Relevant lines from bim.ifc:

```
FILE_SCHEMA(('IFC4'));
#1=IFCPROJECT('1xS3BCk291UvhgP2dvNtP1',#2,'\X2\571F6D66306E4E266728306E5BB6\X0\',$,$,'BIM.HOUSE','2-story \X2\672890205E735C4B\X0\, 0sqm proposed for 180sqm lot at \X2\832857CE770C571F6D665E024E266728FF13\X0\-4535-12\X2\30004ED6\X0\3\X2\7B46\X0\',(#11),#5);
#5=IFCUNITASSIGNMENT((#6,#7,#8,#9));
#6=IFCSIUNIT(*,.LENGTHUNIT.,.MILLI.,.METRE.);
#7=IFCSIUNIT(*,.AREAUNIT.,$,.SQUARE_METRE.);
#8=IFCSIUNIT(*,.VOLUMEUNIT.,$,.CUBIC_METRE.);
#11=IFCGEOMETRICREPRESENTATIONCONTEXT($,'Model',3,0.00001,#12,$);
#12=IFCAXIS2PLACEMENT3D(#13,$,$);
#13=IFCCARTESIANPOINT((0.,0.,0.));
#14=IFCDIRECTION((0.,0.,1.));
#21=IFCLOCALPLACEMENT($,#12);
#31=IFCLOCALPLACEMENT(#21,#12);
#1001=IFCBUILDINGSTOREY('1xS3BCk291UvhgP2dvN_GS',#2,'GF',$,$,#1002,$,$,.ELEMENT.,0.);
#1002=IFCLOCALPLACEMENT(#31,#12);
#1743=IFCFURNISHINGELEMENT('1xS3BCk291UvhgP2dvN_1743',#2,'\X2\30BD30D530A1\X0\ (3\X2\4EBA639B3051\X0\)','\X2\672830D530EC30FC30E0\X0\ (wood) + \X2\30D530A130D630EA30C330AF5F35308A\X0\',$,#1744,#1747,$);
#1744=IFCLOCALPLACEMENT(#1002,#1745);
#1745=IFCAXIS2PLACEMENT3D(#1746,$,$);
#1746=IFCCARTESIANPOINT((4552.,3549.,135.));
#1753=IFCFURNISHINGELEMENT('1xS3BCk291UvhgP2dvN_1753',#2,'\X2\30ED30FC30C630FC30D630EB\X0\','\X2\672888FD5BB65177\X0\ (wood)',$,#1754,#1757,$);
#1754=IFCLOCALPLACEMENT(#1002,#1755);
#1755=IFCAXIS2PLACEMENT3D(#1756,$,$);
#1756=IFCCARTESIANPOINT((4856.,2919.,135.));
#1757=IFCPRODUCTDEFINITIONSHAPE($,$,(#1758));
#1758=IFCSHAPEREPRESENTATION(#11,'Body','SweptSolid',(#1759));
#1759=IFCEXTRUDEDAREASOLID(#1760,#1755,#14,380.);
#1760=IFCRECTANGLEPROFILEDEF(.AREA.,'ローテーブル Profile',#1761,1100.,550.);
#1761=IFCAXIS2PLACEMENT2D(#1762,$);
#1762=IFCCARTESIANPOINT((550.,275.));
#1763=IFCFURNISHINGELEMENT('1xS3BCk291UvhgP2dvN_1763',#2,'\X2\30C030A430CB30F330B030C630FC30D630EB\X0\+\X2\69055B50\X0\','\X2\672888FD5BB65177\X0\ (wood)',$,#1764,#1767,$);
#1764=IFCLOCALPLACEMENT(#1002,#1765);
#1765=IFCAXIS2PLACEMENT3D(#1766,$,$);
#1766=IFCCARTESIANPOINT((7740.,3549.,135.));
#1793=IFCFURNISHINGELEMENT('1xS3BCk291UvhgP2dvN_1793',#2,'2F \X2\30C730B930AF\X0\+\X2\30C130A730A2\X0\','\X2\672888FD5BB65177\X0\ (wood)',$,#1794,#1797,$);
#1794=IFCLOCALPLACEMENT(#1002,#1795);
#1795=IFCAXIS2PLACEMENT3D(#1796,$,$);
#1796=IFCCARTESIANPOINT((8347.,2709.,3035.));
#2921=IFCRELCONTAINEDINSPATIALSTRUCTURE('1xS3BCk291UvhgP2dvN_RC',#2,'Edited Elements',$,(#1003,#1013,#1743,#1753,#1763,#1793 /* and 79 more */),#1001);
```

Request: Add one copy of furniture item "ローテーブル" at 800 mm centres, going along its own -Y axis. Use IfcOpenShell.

```python
import ifcopenshell
import ifcopenshell.api.geometry
import ifcopenshell.api.root
import ifcopenshell.util.element
import ifcopenshell.util.placement
import ifcopenshell.util.unit

model = ifcopenshell.open("bim.ifc")
unit_scale = ifcopenshell.util.unit.calculate_unit_scale(model)


def reuse_history(source, copy):
    """copy_class also copies each property set's owner history, people and application; keep the originals."""
    for rel in copy.IsDefinedBy:
        if rel.is_a("IfcRelDefinesByProperties") and (history := rel.RelatingPropertyDefinition.OwnerHistory):
            rel.RelatingPropertyDefinition.OwnerHistory = source.OwnerHistory
            ifcopenshell.util.element.remove_deep2(model, history)


source = model.by_guid("1xS3BCk291UvhgP2dvN_1753")
base = ifcopenshell.util.placement.get_local_placement(source.ObjectPlacement)
step = -base[:3, 1] * 0.8 / unit_scale

for i in range(1, 2):
    copy = ifcopenshell.api.root.copy_class(model, product=source)
    copy.Representation = ifcopenshell.util.element.copy_deep(
        model, source.Representation, exclude=["IfcGeometricRepresentationContext", "IfcRepresentationMap"]
    )
    reuse_history(source, copy)
    matrix = base.copy()
    matrix[:3, 3] += i * step
    print("added at", matrix[:3, 3].round(3) + 0.0)
    ifcopenshell.api.geometry.edit_object_placement(model, product=copy, matrix=matrix, is_si=False)

model.write("bim_updated.ifc")
```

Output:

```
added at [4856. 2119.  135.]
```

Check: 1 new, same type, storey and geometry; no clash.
